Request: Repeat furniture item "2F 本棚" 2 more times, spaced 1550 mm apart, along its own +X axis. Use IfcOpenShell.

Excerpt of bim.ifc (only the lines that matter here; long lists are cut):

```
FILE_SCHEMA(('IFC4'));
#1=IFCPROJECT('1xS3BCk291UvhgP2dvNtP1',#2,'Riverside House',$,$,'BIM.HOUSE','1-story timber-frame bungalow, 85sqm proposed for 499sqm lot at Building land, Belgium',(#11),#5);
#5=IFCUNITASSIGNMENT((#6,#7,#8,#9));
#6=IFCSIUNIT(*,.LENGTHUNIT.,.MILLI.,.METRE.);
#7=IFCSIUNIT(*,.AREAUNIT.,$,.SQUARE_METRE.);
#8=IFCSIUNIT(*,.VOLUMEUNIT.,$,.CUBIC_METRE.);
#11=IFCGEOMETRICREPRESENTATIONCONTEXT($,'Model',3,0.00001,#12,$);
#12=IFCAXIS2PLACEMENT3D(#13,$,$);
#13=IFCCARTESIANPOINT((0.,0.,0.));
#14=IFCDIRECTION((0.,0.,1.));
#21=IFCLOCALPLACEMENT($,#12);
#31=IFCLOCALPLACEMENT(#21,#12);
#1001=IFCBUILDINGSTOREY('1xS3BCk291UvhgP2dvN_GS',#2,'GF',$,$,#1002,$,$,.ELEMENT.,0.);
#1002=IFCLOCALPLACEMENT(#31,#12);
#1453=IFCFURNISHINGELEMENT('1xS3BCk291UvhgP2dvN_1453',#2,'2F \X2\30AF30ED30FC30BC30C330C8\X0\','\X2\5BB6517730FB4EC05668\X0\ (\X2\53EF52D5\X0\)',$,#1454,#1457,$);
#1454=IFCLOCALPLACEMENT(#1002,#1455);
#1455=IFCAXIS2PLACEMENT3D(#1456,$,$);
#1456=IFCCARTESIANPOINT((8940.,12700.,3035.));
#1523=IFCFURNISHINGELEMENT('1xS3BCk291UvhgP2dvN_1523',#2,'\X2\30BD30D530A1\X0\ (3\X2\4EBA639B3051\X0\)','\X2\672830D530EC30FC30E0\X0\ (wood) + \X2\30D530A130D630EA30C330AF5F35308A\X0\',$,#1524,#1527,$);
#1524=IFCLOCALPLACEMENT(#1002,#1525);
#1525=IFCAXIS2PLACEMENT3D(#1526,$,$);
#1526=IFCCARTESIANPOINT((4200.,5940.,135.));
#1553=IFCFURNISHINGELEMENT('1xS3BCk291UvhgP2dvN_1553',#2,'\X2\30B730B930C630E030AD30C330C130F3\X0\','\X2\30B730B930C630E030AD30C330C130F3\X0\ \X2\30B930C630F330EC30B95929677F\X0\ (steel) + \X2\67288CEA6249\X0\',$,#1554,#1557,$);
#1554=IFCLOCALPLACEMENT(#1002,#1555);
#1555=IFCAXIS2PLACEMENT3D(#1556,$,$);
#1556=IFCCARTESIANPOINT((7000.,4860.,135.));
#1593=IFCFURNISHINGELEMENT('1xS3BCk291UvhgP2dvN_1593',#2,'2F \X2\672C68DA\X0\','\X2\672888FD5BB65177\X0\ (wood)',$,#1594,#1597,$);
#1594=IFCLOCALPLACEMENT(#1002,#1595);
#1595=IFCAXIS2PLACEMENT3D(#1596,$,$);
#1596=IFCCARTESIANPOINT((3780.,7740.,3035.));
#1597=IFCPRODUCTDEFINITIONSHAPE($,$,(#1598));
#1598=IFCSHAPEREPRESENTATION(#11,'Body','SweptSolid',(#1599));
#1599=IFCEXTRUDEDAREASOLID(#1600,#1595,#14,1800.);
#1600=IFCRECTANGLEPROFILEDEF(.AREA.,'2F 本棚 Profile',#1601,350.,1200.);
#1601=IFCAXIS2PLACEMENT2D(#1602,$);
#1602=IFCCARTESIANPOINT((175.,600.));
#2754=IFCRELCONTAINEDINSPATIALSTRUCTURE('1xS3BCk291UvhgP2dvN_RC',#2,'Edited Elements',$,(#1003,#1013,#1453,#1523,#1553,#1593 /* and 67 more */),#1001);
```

```python
import ifcopenshell
import ifcopenshell.api.geometry
import ifcopenshell.api.root
import ifcopenshell.util.element
import ifcopenshell.util.placement

model = ifcopenshell.open("bim.ifc")


def reuse_history(source, copy):
    """copy_class also copies each property set's owner history, people and application; keep the originals."""
    for rel in copy.IsDefinedBy:
        if rel.is_a("IfcRelDefinesByProperties") and (history := rel.RelatingPropertyDefinition.OwnerHistory):
            rel.RelatingPropertyDefinition.OwnerHistory = source.OwnerHistory
            ifcopenshell.util.element.remove_deep2(model, history)


source = model.by_guid("1xS3BCk291UvhgP2dvN_1593")
base = ifcopenshell.util.placement.get_local_placement(source.ObjectPlacement)
step = base[:3, 0] * 1550.0

for i in range(1, 3):
    copy = ifcopenshell.api.root.copy_class(model, product=source)
    copy.Representation = ifcopenshell.util.element.copy_deep(
        model, source.Representation, exclude=["IfcGeometricRepresentationContext", "IfcRepresentationMap"]
    )
    reuse_history(source, copy)
    matrix = base.copy()
    matrix[:3, 3] += i * step
    print("added at", matrix[:3, 3].round(3) + 0.0)
    ifcopenshell.api.geometry.edit_object_placement(model, product=copy, matrix=matrix, is_si=False)

model.write("bim_edited.ifc")
```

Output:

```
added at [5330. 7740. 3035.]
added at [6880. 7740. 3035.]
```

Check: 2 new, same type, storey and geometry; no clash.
